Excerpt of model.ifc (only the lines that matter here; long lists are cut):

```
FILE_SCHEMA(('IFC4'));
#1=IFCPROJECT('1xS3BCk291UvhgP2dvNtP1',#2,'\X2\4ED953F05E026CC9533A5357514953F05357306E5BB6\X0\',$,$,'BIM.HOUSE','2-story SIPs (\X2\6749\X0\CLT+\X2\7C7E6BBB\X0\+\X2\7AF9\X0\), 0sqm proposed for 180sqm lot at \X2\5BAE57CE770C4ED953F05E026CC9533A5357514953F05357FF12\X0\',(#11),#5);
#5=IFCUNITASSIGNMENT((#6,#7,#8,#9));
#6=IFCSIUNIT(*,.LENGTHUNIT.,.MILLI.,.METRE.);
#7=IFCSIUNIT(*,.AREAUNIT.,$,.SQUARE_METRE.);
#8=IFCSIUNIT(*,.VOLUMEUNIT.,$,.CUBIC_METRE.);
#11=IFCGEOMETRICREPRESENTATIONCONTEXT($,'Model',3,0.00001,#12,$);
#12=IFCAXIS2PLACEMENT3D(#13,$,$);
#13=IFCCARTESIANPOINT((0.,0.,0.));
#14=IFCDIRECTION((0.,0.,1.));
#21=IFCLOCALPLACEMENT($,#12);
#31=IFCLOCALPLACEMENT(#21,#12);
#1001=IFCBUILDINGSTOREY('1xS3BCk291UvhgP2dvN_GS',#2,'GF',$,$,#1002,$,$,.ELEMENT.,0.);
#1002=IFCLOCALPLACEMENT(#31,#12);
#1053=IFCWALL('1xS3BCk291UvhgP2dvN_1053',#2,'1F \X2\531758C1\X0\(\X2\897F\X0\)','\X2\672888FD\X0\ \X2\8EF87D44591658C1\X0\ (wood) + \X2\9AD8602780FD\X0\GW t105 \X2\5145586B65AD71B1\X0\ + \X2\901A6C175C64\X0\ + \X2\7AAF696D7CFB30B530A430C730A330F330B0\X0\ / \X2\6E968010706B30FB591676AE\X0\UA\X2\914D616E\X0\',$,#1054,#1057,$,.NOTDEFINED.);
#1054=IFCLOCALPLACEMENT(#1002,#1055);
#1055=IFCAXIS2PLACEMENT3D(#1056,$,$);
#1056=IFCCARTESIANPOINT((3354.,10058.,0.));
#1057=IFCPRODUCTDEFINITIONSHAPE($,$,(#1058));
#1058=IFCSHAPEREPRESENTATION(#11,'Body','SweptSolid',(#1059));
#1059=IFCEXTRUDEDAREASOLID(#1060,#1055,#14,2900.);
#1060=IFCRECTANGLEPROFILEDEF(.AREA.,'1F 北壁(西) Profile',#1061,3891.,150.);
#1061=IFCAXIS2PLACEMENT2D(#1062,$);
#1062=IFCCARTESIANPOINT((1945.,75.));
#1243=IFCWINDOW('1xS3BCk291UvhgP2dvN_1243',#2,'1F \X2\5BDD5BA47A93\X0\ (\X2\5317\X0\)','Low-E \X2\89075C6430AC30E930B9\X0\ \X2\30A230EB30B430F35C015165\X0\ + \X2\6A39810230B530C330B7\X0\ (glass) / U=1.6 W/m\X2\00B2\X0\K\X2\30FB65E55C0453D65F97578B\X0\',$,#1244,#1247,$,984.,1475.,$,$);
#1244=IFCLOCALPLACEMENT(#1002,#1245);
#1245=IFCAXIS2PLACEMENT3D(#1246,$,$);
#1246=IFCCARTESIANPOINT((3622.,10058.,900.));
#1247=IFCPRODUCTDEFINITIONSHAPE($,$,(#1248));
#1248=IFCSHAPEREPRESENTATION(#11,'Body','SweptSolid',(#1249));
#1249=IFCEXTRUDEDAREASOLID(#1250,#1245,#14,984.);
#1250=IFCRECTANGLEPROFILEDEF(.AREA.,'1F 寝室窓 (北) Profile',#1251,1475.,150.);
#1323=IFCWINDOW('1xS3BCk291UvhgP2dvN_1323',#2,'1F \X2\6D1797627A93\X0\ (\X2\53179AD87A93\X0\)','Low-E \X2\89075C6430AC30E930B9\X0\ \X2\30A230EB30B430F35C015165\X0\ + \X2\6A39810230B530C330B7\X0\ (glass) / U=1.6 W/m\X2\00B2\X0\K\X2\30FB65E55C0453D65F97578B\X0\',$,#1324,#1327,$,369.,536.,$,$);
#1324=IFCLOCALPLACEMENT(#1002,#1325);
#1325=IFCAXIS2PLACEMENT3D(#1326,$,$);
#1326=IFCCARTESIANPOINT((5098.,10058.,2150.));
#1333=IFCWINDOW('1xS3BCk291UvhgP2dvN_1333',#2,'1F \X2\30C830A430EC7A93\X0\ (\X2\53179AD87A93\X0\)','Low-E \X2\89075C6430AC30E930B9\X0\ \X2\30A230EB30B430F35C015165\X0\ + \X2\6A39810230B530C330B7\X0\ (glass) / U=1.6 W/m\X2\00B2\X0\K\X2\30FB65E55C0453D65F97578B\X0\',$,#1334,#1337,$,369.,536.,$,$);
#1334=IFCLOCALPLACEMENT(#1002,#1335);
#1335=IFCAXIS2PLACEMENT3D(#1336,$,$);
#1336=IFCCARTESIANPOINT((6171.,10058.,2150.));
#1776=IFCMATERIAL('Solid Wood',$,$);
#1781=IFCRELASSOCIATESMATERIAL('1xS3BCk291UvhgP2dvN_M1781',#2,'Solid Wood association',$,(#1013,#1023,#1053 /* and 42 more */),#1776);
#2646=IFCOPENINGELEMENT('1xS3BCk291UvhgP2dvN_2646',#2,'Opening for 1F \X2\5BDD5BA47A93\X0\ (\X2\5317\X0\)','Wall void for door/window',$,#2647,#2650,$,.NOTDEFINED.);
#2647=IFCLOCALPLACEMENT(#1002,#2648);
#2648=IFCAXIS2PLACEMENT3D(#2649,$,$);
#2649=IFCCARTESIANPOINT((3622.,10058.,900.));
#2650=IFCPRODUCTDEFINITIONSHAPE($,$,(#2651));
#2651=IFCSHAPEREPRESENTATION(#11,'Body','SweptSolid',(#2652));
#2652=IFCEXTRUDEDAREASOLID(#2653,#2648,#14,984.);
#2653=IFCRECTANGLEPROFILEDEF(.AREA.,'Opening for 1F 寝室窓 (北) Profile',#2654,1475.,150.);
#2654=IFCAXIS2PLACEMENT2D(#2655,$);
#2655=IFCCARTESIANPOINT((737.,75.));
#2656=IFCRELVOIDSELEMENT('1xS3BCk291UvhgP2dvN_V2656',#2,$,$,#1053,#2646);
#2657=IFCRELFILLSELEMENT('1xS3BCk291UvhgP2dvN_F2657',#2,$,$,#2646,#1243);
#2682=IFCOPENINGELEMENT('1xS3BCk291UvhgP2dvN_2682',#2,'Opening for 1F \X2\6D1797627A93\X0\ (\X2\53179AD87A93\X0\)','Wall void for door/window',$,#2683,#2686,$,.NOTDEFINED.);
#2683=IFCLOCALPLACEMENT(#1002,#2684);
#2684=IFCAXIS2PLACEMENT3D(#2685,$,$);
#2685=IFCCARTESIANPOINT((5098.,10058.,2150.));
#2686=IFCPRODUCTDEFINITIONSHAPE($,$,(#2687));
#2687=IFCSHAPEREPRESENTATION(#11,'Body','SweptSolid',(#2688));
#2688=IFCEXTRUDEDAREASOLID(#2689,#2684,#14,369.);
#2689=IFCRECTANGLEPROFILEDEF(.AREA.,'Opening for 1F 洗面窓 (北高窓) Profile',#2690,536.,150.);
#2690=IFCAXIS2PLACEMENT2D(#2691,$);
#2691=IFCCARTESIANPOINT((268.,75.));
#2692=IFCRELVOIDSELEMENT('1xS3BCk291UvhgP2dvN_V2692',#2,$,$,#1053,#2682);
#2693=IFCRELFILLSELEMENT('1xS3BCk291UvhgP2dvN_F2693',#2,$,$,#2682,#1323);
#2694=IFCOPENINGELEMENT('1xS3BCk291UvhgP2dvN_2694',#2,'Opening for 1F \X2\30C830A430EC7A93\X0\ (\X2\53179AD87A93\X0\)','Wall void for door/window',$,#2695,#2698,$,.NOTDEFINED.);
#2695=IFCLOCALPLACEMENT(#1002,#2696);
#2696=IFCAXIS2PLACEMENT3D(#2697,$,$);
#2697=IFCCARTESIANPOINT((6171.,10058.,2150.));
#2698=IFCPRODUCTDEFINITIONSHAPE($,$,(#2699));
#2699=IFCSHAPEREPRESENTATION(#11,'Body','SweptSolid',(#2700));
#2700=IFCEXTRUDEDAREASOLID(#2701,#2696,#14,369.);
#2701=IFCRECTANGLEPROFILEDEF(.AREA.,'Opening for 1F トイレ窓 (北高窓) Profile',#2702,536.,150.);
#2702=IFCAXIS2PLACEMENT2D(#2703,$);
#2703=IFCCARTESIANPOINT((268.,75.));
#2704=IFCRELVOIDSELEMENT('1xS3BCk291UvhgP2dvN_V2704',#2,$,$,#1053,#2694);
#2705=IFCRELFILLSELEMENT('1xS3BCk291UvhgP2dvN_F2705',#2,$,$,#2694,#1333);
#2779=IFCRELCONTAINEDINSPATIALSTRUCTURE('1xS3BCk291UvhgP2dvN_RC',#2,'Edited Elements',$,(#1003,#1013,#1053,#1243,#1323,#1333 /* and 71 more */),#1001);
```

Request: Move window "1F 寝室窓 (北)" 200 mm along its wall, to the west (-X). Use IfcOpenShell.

```python
import ifcopenshell
import ifcopenshell.api.geometry
import ifcopenshell.util.placement

model = ifcopenshell.open("model.ifc")

window = model.by_guid("1xS3BCk291UvhgP2dvN_1243")
opening = window.FillsVoids[0].RelatingOpeningElement
wall = opening.VoidsElements[0].RelatingBuildingElement

wall_matrix = ifcopenshell.util.placement.get_local_placement(wall.ObjectPlacement)
shift = wall_matrix[:3, 0] * -200.0
before = ifcopenshell.util.placement.get_local_placement(window.ObjectPlacement)[:3, 3].copy()

# The window is not placed relative to its opening, so move both.
for product in (opening, window):
    matrix = ifcopenshell.util.placement.get_local_placement(product.ObjectPlacement)
    matrix[:3, 3] += shift
    ifcopenshell.api.geometry.edit_object_placement(model, product=product, matrix=matrix, is_si=False)

after = ifcopenshell.util.placement.get_local_placement(window.ObjectPlacement)[:3, 3]
print("window moved by", (after - before).round(3) + 0.0)

model.write("model_v2.ifc")
```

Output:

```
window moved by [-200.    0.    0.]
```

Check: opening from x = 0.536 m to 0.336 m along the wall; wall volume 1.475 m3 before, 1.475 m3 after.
